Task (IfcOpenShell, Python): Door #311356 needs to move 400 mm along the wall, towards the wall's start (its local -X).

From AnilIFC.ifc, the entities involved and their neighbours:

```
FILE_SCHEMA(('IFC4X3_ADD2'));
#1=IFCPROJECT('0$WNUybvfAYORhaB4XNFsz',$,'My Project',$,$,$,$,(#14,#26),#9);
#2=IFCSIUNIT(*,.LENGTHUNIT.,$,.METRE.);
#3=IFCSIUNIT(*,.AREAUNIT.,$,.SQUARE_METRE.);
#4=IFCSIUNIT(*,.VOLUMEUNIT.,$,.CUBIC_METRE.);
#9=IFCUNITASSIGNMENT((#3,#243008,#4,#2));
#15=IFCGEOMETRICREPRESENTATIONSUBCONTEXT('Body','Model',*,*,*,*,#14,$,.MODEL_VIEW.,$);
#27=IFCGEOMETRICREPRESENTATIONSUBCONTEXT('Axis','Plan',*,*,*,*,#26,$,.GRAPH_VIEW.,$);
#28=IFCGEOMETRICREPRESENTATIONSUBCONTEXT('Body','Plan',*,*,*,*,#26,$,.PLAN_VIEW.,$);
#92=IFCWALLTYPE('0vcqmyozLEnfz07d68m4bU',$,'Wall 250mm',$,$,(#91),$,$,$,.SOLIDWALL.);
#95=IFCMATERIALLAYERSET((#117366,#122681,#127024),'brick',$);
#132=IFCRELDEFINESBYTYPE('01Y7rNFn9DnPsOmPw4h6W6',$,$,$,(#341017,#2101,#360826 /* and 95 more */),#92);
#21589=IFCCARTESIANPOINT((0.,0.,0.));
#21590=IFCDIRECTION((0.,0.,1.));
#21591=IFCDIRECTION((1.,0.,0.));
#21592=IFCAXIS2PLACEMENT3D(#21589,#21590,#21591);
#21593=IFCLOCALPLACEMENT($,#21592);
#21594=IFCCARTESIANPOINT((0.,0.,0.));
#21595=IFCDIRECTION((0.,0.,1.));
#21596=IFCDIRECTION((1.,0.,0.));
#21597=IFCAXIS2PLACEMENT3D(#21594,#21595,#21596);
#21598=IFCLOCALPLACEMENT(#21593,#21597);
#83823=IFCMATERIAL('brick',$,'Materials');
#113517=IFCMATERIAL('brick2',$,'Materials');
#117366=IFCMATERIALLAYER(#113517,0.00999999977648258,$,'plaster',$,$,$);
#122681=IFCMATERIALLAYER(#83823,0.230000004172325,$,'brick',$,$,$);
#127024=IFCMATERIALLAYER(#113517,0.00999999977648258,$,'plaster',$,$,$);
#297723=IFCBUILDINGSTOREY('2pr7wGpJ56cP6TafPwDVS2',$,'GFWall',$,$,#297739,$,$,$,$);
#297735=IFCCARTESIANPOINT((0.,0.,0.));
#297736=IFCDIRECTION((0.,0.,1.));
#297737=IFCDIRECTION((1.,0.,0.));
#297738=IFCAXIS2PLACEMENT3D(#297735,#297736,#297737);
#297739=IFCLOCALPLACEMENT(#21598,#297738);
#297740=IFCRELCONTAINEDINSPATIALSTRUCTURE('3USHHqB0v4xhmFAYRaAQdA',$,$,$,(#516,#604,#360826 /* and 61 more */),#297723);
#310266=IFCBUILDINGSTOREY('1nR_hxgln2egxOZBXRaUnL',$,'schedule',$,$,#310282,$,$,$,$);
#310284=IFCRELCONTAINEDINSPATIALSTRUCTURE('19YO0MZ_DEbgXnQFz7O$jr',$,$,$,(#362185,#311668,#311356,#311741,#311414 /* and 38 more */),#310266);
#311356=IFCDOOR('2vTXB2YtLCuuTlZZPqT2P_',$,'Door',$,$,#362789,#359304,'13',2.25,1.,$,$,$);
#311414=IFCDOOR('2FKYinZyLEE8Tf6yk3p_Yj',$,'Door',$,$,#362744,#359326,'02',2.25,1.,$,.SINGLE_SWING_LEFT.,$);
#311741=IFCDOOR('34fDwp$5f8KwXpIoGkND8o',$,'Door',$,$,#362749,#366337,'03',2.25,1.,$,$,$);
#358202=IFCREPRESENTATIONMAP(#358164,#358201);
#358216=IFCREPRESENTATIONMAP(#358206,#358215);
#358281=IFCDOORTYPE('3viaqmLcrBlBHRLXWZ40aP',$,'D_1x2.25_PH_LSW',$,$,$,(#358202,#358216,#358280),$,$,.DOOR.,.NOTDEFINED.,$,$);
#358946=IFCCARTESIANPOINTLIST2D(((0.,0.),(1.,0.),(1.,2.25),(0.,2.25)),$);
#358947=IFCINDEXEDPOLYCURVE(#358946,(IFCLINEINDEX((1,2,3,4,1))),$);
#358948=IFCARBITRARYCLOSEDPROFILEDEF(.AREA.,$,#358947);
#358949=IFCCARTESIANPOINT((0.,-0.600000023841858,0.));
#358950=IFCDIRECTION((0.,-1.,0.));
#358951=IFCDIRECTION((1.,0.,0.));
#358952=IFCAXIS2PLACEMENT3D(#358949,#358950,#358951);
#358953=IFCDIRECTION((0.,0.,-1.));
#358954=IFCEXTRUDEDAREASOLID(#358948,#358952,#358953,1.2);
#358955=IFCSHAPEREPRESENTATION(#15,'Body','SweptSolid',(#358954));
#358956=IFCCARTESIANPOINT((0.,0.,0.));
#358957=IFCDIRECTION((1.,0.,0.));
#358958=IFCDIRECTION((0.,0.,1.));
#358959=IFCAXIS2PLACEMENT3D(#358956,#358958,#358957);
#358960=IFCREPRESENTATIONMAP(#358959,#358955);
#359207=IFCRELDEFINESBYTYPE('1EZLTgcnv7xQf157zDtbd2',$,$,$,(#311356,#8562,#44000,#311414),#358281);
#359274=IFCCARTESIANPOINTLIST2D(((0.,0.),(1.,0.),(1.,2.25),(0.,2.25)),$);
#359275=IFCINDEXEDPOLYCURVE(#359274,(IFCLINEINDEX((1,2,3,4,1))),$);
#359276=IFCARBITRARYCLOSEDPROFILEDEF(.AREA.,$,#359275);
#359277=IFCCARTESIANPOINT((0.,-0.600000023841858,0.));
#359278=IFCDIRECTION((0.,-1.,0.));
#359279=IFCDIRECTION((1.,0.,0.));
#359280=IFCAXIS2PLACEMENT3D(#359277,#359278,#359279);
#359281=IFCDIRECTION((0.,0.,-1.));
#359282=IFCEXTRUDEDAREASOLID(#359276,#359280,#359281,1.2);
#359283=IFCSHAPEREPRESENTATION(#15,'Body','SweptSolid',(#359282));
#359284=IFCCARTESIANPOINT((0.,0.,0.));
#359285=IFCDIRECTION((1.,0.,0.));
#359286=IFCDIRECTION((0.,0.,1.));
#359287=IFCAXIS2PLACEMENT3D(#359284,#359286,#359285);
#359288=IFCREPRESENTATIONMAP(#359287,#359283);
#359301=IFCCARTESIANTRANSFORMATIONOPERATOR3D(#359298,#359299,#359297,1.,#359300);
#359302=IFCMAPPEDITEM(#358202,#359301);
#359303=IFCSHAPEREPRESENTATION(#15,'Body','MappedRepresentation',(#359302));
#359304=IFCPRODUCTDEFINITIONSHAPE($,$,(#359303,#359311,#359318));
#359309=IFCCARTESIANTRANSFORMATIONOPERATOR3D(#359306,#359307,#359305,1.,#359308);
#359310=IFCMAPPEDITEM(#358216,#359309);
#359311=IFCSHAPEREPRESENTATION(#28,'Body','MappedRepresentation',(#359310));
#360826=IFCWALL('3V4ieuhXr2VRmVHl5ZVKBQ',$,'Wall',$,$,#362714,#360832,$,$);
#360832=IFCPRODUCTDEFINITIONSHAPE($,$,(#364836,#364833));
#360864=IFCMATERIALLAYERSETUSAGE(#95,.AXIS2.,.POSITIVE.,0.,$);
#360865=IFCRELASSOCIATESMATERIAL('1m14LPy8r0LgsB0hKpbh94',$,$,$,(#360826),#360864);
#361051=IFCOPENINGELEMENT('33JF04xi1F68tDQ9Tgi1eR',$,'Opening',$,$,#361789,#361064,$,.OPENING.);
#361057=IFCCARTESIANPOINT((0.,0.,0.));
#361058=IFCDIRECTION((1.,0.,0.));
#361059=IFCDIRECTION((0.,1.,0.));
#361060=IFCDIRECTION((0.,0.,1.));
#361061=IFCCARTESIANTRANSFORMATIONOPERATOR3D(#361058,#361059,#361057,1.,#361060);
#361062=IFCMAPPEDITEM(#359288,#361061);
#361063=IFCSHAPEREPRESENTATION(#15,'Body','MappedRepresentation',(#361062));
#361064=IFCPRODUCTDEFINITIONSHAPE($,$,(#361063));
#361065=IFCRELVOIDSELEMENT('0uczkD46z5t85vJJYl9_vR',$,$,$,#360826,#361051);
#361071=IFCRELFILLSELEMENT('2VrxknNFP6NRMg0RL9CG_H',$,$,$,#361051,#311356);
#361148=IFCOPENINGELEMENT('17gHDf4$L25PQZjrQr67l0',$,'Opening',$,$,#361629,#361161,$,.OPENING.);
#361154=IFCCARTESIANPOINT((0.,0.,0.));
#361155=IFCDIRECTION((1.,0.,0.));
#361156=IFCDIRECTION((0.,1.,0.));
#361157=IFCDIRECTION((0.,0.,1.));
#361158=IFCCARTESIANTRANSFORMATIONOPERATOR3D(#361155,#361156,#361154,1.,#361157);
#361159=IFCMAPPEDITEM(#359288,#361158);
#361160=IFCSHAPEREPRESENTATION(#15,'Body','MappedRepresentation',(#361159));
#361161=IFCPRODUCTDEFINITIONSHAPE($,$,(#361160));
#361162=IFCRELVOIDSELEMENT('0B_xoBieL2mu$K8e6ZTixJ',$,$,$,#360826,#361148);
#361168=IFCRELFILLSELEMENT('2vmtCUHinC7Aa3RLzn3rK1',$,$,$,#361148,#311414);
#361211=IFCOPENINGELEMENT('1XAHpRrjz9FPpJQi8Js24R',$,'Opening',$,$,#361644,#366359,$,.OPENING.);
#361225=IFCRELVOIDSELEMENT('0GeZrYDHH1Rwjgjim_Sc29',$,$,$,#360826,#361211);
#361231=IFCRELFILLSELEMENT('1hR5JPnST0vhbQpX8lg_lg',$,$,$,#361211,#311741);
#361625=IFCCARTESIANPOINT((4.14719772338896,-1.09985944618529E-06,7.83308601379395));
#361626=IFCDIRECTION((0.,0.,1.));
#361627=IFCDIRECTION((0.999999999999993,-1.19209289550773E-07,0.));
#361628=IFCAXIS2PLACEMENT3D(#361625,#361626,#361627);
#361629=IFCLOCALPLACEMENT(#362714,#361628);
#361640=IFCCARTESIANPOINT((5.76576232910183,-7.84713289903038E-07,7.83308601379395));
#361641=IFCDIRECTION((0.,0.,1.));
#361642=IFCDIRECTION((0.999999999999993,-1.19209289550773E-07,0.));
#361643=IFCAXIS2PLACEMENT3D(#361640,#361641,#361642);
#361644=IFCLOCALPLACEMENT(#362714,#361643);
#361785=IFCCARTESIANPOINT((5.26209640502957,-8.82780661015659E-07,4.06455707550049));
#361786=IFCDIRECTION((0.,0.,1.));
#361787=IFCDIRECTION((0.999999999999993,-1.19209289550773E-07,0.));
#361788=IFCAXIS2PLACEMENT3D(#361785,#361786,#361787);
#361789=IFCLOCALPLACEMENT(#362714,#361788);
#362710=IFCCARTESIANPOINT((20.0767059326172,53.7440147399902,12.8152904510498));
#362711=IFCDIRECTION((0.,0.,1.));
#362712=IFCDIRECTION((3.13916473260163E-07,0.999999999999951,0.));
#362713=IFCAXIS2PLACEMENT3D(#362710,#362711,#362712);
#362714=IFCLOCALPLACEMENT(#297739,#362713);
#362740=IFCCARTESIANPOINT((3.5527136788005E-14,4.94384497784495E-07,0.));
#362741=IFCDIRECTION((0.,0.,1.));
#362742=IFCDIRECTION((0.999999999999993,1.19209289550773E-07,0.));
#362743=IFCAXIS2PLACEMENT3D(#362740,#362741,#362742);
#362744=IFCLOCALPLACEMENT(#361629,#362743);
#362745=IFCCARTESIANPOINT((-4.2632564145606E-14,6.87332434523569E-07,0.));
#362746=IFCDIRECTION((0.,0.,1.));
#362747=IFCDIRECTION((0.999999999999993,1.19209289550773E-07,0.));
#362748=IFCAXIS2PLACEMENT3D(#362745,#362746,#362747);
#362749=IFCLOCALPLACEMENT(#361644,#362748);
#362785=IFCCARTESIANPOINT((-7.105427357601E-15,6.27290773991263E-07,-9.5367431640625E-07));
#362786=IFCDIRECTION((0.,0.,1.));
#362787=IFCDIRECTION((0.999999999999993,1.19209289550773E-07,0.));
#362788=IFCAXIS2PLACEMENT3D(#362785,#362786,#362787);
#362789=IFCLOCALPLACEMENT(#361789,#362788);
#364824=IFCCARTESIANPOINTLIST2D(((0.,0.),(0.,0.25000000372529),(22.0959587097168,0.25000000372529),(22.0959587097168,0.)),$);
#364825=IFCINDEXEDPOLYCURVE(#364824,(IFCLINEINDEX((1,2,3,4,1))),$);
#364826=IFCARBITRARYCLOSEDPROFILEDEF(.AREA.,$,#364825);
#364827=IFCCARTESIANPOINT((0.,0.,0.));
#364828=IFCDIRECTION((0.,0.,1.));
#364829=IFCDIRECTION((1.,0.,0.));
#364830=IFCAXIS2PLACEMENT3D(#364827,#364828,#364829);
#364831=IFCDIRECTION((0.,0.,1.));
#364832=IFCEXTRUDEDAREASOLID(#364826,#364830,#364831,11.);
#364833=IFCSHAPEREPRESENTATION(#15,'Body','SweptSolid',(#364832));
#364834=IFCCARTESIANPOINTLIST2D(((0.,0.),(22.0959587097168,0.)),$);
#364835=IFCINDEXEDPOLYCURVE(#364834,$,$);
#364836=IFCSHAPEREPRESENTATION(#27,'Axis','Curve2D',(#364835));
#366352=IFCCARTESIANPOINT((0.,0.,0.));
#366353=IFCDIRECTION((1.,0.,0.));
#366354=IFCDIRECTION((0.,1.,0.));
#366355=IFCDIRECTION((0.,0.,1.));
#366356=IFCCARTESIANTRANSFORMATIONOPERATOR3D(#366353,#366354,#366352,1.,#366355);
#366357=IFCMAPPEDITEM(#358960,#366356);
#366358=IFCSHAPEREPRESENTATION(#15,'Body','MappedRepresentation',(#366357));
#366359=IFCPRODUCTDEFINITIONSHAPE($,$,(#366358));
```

```python
import ifcopenshell
import ifcopenshell.api.geometry
import ifcopenshell.util.placement

model = ifcopenshell.open("AnilIFC.ifc")

door = model.by_id(311356)
opening = door.FillsVoids[0].RelatingOpeningElement
wall = opening.VoidsElements[0].RelatingBuildingElement

wall_matrix = ifcopenshell.util.placement.get_local_placement(wall.ObjectPlacement)
shift = wall_matrix[:3, 0] * -0.4
before = ifcopenshell.util.placement.get_local_placement(door.ObjectPlacement)[:3, 3].copy()

# The door is placed relative to its opening, so it follows when the opening moves.
matrix = ifcopenshell.util.placement.get_local_placement(opening.ObjectPlacement)
matrix[:3, 3] += shift
ifcopenshell.api.geometry.edit_object_placement(
    model, product=opening, matrix=matrix, is_si=False, should_transform_children=True
)

after = ifcopenshell.util.placement.get_local_placement(door.ObjectPlacement)[:3, 3]
print("door moved by", (after - before).round(3) + 0.0)

model.write("AnilIFC_updated.ifc")
```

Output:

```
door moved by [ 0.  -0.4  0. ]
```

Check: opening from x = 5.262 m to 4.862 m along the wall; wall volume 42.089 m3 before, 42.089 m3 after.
